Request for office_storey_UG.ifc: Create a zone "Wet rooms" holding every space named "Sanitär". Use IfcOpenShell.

First a look at what the model holds.

```python
import ifcopenshell

model = ifcopenshell.open("office_storey_UG.ifc")
print(model.schema)
seen = {}
for space in model.by_type("IfcSpace"):
    seen[space.LongName] = seen.get(space.LongName, 0) + 1
for name, count in sorted(seen.items(), key=str):
    print(count, "x", name)
print("zones:", [z.Name for z in model.by_type("IfcZone")][:20])
```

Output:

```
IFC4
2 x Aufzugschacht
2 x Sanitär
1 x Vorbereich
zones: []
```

```python
import ifcopenshell
import ifcopenshell.api.group
import ifcopenshell.api.root

model = ifcopenshell.open("office_storey_UG.ifc")

names = {"Sanitär"}
spaces = [s for s in model.by_type("IfcSpace") if s.LongName in names]

zone = ifcopenshell.api.root.create_entity(model, ifc_class="IfcZone", name="Wet rooms")
ifcopenshell.api.group.assign_group(model, products=spaces, group=zone)
print(len(spaces), "spaces in", zone.Name)

model.write("office_storey_UG_v2.ifc")
```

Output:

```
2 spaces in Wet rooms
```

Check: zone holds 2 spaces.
